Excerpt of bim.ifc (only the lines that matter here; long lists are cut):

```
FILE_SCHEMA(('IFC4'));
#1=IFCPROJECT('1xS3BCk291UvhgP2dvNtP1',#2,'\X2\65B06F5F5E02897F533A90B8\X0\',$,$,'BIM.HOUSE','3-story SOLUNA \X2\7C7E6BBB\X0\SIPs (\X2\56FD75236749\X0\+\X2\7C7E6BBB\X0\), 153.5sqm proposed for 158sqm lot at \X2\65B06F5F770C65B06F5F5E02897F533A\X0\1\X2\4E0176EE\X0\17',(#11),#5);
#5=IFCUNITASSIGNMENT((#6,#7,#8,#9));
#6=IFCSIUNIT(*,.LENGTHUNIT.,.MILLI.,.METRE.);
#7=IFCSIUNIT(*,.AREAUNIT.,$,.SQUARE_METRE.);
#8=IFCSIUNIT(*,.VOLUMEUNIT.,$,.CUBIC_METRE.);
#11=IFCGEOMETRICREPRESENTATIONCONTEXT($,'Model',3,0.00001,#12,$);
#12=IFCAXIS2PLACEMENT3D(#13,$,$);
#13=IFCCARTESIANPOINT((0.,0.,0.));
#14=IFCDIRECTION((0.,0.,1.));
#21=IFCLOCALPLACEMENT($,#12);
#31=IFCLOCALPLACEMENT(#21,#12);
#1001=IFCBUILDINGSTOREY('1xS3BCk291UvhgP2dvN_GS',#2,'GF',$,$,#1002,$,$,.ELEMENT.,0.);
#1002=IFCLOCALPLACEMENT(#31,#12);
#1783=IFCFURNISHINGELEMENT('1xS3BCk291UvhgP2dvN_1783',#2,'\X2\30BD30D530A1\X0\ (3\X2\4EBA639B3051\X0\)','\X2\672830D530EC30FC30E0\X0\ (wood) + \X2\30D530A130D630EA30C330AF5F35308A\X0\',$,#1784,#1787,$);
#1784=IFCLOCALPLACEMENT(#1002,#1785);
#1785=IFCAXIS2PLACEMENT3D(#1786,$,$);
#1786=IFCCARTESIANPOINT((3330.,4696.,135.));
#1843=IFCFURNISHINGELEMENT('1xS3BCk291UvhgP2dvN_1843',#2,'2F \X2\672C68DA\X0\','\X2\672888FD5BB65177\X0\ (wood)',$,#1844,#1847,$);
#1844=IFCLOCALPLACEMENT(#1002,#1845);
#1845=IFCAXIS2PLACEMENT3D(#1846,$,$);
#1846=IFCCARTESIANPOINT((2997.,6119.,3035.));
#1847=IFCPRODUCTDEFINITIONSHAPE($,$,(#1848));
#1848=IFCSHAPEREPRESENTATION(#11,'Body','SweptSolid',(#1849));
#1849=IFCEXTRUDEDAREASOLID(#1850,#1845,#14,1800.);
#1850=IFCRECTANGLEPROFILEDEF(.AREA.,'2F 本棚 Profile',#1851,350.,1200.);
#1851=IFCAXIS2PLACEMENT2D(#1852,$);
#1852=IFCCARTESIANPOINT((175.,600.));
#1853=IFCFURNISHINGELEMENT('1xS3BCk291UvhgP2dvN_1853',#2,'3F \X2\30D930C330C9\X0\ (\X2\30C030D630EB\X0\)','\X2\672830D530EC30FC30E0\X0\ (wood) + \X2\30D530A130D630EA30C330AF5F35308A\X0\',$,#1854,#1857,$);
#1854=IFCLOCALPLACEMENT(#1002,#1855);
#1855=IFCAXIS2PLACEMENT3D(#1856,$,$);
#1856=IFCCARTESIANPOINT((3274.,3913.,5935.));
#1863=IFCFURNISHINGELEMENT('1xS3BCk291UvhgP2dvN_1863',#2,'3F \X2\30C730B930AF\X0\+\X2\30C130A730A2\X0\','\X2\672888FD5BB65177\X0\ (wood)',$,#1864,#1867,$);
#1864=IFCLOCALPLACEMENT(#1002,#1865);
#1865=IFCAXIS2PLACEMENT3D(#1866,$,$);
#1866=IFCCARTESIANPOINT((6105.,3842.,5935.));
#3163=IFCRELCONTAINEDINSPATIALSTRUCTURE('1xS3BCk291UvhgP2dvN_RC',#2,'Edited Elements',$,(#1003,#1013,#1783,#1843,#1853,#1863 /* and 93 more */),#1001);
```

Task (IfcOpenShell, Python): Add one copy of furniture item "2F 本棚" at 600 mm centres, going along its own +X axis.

```python
import ifcopenshell
import ifcopenshell.api.geometry
import ifcopenshell.api.root
import ifcopenshell.util.element
import ifcopenshell.util.placement
import ifcopenshell.util.unit

model = ifcopenshell.open("bim.ifc")
unit_scale = ifcopenshell.util.unit.calculate_unit_scale(model)


def reuse_history(source, copy):
    """copy_class also copies each property set's owner history, people and application; keep the originals."""
    for rel in copy.IsDefinedBy:
        if rel.is_a("IfcRelDefinesByProperties") and (history := rel.RelatingPropertyDefinition.OwnerHistory):
            rel.RelatingPropertyDefinition.OwnerHistory = source.OwnerHistory
            ifcopenshell.util.element.remove_deep2(model, history)


source = model.by_guid("1xS3BCk291UvhgP2dvN_1843")
base = ifcopenshell.util.placement.get_local_placement(source.ObjectPlacement)
step = base[:3, 0] * 0.6 / unit_scale

for i in range(1, 2):
    copy = ifcopenshell.api.root.copy_class(model, product=source)
    copy.Representation = ifcopenshell.util.element.copy_deep(
        model, source.Representation, exclude=["IfcGeometricRepresentationContext", "IfcRepresentationMap"]
    )
    reuse_history(source, copy)
    matrix = base.copy()
    matrix[:3, 3] += i * step
    print("added at", matrix[:3, 3].round(3) + 0.0)
    ifcopenshell.api.geometry.edit_object_placement(model, product=copy, matrix=matrix, is_si=False)

model.write("bim_updated.ifc")
```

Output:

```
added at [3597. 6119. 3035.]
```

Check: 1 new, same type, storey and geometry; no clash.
